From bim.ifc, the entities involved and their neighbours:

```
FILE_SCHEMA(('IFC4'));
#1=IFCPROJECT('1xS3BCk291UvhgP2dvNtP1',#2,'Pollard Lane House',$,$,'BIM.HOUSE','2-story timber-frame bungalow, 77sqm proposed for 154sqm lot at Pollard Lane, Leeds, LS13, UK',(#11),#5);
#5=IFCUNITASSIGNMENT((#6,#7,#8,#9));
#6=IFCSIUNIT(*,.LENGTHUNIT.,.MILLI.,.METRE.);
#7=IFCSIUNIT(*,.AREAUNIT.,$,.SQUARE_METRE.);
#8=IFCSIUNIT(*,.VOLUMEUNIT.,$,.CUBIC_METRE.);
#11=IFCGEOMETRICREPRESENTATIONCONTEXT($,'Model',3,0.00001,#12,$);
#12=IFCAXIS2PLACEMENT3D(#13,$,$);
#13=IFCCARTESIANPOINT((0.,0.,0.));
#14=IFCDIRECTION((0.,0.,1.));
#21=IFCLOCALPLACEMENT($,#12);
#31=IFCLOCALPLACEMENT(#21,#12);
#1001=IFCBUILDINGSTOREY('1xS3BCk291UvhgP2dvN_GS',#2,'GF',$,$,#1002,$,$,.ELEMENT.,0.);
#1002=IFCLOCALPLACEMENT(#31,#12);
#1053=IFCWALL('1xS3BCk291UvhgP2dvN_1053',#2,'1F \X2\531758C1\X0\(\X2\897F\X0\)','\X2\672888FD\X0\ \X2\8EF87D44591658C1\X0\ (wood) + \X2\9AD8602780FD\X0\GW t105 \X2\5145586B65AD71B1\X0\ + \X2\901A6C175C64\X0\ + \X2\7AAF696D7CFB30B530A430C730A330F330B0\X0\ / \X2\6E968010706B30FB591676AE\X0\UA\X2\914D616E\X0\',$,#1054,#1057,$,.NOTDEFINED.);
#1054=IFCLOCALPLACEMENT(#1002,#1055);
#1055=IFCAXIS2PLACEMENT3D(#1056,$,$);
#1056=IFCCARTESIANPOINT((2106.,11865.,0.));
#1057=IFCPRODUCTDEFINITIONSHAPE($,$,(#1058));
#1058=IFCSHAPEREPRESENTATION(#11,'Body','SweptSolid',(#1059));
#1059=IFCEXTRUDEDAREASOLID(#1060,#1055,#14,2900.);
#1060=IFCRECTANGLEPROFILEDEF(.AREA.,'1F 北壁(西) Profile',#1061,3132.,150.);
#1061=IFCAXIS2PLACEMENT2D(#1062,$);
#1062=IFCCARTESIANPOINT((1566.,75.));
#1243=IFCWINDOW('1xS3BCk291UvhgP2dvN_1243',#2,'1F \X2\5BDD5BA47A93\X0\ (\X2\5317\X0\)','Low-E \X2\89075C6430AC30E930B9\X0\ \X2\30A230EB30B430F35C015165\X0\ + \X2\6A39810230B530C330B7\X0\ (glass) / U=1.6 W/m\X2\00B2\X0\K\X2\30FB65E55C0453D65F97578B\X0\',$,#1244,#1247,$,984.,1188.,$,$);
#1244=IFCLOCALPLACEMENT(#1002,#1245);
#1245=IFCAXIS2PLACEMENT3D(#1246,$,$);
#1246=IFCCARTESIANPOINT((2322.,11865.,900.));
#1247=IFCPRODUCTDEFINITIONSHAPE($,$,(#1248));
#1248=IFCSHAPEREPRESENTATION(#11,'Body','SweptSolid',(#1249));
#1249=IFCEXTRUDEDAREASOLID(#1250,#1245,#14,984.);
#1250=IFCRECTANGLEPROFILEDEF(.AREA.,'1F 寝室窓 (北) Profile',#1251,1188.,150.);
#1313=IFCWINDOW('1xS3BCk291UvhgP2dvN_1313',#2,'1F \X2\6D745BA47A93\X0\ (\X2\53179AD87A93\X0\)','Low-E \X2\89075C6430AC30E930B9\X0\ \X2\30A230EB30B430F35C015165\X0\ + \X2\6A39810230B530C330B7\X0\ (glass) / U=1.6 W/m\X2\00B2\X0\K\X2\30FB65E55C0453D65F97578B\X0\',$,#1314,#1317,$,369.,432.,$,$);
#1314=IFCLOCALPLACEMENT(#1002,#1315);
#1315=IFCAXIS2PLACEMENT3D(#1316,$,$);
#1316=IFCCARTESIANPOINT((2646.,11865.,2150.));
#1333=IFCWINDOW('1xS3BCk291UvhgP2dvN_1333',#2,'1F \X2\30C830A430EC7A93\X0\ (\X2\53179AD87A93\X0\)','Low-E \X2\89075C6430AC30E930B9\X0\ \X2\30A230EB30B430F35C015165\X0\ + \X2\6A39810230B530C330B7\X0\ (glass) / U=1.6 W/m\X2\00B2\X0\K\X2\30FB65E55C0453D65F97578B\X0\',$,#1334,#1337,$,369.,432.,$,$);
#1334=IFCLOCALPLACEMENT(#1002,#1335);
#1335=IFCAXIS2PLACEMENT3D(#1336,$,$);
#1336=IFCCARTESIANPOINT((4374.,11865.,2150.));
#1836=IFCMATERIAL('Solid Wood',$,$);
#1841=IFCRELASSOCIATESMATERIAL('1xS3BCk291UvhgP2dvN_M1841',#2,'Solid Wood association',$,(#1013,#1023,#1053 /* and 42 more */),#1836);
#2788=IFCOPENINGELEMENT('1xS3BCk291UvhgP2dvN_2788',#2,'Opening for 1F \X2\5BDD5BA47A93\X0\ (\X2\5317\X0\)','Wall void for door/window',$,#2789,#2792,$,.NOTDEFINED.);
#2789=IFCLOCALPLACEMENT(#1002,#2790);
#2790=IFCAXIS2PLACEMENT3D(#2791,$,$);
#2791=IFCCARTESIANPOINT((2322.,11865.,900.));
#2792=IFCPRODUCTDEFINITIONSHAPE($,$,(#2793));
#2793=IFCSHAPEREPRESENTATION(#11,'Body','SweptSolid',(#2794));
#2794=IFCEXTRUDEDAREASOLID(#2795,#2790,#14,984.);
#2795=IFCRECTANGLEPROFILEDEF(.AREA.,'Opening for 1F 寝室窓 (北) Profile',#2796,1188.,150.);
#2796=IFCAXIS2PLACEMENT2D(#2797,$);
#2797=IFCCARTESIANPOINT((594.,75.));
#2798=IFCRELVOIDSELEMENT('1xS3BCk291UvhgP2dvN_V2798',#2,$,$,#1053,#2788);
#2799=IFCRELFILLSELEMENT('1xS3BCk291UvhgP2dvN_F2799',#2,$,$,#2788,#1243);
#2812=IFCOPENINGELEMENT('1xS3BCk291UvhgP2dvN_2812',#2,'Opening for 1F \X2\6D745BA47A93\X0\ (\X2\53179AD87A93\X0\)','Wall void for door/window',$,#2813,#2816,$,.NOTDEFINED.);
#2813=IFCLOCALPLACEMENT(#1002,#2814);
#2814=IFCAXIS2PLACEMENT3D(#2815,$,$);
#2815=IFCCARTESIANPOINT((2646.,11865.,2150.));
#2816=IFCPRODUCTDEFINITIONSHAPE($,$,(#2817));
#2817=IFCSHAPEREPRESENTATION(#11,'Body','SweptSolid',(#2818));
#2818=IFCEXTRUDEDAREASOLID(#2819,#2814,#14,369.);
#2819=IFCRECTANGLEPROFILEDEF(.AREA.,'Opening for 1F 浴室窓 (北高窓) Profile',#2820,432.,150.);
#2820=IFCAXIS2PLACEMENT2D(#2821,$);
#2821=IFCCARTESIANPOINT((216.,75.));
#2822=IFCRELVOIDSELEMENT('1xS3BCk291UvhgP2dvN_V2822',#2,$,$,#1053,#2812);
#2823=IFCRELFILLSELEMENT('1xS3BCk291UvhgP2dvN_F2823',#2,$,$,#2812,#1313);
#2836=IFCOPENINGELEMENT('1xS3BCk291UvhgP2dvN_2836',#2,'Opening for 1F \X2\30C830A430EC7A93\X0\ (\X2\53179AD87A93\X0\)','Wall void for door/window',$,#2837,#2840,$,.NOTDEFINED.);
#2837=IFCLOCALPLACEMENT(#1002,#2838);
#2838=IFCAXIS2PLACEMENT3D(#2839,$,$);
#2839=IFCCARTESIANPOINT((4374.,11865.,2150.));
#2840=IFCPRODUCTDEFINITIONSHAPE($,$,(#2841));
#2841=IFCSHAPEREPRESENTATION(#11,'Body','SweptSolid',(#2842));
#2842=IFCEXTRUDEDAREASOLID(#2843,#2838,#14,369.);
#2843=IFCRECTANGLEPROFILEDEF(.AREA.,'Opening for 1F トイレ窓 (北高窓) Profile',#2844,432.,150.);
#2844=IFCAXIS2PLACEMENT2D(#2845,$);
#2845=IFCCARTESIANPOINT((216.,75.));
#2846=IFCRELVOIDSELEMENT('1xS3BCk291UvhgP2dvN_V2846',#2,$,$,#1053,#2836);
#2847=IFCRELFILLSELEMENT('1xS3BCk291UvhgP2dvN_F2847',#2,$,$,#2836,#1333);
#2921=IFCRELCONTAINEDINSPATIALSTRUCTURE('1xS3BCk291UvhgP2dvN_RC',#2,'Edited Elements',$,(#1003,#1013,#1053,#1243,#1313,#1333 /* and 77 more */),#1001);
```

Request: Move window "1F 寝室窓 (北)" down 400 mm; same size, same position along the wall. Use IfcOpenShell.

```python
import numpy as np
import ifcopenshell
import ifcopenshell.api.geometry
import ifcopenshell.util.placement
import ifcopenshell.util.unit

model = ifcopenshell.open("bim.ifc")
unit_scale = ifcopenshell.util.unit.calculate_unit_scale(model)

window = model.by_id(1243)
opening = window.FillsVoids[0].RelatingOpeningElement
dz = -0.4 / unit_scale

shift = np.array([0.0, 0.0, dz])
# The window is not placed relative to its opening, so move both.
for product in (opening, window):
    matrix = ifcopenshell.util.placement.get_local_placement(product.ObjectPlacement)
    matrix[:3, 3] += shift
    ifcopenshell.api.geometry.edit_object_placement(model, product=product, matrix=matrix, is_si=False)

print(f"moved by {dz * unit_scale:+.3f} m")

model.write("bim-out.ifc")
```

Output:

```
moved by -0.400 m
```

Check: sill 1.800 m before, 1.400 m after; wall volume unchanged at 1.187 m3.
